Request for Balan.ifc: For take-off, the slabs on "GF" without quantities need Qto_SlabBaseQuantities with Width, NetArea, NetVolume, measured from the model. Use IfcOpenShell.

First a look at what the model holds.

```python
import ifcopenshell
import ifcopenshell.util.element
import ifcopenshell.util.unit

model = ifcopenshell.open("Balan.ifc")
print(model.schema)
for unit_type in ("LENGTHUNIT", "AREAUNIT", "VOLUMEUNIT"):
    print(unit_type, ifcopenshell.util.unit.calculate_unit_scale(model, unit_type))
storey = next(s for s in model.by_type("IfcBuildingStorey") if s.Name == "GF")
slabs = [e for e in ifcopenshell.util.element.get_decomposition(storey) if e.is_a("IfcSlab")]
for e in sorted(slabs, key=lambda e: e.id()):
    print(e.id(), e.is_a(), e.Name, list(ifcopenshell.util.element.get_psets(e, qtos_only=True)), sep=" | ")
```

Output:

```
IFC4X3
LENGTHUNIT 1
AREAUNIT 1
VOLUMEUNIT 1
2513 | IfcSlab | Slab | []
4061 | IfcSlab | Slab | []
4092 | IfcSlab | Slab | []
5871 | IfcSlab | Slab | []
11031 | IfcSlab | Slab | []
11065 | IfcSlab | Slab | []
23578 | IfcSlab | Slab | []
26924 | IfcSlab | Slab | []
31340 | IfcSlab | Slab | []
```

```python
import ifcopenshell
import ifcopenshell.api.pset
import ifcopenshell.geom
import ifcopenshell.util.element
import ifcopenshell.util.shape
import ifcopenshell.util.unit

model = ifcopenshell.open("Balan.ifc")
unit_scale = ifcopenshell.util.unit.calculate_unit_scale(model)
area_scale = ifcopenshell.util.unit.calculate_unit_scale(model, "AREAUNIT")
volume_scale = ifcopenshell.util.unit.calculate_unit_scale(model, "VOLUMEUNIT")
settings = ifcopenshell.geom.settings()

storey = next(s for s in model.by_type("IfcBuildingStorey") if s.Name == "GF")
slabs = [e for e in ifcopenshell.util.element.get_decomposition(storey) if e.is_a("IfcSlab")]

for e in sorted(slabs, key=lambda e: e.id()):
    if ifcopenshell.util.element.get_psets(e, qtos_only=True, should_inherit=False):
        continue
    # Geometry comes back in metres, in the element's own axes.
    shape = ifcopenshell.geom.create_shape(settings, e)
    values = {
        "Width": ifcopenshell.util.shape.get_z(shape.geometry) / unit_scale,
        "NetArea": ifcopenshell.util.shape.get_footprint_area(shape.geometry) / area_scale,
        "NetVolume": ifcopenshell.util.shape.get_volume(shape.geometry) / volume_scale,
    }
    qto = ifcopenshell.api.pset.add_qto(model, product=e, name="Qto_SlabBaseQuantities")
    ifcopenshell.api.pset.edit_qto(model, qto=qto, properties=values)
    print(e.id(), {k: round(v, 3) for k, v in values.items()})

model.write("Balan_rev.ifc")
```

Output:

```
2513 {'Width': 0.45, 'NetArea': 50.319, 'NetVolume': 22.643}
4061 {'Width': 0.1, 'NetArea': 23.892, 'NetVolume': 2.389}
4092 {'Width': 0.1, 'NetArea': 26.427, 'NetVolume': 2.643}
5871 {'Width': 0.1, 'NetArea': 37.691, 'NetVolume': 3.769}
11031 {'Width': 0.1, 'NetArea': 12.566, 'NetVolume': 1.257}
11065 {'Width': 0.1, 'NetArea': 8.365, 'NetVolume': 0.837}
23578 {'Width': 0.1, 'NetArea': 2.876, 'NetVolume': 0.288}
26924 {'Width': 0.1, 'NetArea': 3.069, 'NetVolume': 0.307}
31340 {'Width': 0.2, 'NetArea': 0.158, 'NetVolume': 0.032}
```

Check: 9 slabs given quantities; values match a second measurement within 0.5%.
